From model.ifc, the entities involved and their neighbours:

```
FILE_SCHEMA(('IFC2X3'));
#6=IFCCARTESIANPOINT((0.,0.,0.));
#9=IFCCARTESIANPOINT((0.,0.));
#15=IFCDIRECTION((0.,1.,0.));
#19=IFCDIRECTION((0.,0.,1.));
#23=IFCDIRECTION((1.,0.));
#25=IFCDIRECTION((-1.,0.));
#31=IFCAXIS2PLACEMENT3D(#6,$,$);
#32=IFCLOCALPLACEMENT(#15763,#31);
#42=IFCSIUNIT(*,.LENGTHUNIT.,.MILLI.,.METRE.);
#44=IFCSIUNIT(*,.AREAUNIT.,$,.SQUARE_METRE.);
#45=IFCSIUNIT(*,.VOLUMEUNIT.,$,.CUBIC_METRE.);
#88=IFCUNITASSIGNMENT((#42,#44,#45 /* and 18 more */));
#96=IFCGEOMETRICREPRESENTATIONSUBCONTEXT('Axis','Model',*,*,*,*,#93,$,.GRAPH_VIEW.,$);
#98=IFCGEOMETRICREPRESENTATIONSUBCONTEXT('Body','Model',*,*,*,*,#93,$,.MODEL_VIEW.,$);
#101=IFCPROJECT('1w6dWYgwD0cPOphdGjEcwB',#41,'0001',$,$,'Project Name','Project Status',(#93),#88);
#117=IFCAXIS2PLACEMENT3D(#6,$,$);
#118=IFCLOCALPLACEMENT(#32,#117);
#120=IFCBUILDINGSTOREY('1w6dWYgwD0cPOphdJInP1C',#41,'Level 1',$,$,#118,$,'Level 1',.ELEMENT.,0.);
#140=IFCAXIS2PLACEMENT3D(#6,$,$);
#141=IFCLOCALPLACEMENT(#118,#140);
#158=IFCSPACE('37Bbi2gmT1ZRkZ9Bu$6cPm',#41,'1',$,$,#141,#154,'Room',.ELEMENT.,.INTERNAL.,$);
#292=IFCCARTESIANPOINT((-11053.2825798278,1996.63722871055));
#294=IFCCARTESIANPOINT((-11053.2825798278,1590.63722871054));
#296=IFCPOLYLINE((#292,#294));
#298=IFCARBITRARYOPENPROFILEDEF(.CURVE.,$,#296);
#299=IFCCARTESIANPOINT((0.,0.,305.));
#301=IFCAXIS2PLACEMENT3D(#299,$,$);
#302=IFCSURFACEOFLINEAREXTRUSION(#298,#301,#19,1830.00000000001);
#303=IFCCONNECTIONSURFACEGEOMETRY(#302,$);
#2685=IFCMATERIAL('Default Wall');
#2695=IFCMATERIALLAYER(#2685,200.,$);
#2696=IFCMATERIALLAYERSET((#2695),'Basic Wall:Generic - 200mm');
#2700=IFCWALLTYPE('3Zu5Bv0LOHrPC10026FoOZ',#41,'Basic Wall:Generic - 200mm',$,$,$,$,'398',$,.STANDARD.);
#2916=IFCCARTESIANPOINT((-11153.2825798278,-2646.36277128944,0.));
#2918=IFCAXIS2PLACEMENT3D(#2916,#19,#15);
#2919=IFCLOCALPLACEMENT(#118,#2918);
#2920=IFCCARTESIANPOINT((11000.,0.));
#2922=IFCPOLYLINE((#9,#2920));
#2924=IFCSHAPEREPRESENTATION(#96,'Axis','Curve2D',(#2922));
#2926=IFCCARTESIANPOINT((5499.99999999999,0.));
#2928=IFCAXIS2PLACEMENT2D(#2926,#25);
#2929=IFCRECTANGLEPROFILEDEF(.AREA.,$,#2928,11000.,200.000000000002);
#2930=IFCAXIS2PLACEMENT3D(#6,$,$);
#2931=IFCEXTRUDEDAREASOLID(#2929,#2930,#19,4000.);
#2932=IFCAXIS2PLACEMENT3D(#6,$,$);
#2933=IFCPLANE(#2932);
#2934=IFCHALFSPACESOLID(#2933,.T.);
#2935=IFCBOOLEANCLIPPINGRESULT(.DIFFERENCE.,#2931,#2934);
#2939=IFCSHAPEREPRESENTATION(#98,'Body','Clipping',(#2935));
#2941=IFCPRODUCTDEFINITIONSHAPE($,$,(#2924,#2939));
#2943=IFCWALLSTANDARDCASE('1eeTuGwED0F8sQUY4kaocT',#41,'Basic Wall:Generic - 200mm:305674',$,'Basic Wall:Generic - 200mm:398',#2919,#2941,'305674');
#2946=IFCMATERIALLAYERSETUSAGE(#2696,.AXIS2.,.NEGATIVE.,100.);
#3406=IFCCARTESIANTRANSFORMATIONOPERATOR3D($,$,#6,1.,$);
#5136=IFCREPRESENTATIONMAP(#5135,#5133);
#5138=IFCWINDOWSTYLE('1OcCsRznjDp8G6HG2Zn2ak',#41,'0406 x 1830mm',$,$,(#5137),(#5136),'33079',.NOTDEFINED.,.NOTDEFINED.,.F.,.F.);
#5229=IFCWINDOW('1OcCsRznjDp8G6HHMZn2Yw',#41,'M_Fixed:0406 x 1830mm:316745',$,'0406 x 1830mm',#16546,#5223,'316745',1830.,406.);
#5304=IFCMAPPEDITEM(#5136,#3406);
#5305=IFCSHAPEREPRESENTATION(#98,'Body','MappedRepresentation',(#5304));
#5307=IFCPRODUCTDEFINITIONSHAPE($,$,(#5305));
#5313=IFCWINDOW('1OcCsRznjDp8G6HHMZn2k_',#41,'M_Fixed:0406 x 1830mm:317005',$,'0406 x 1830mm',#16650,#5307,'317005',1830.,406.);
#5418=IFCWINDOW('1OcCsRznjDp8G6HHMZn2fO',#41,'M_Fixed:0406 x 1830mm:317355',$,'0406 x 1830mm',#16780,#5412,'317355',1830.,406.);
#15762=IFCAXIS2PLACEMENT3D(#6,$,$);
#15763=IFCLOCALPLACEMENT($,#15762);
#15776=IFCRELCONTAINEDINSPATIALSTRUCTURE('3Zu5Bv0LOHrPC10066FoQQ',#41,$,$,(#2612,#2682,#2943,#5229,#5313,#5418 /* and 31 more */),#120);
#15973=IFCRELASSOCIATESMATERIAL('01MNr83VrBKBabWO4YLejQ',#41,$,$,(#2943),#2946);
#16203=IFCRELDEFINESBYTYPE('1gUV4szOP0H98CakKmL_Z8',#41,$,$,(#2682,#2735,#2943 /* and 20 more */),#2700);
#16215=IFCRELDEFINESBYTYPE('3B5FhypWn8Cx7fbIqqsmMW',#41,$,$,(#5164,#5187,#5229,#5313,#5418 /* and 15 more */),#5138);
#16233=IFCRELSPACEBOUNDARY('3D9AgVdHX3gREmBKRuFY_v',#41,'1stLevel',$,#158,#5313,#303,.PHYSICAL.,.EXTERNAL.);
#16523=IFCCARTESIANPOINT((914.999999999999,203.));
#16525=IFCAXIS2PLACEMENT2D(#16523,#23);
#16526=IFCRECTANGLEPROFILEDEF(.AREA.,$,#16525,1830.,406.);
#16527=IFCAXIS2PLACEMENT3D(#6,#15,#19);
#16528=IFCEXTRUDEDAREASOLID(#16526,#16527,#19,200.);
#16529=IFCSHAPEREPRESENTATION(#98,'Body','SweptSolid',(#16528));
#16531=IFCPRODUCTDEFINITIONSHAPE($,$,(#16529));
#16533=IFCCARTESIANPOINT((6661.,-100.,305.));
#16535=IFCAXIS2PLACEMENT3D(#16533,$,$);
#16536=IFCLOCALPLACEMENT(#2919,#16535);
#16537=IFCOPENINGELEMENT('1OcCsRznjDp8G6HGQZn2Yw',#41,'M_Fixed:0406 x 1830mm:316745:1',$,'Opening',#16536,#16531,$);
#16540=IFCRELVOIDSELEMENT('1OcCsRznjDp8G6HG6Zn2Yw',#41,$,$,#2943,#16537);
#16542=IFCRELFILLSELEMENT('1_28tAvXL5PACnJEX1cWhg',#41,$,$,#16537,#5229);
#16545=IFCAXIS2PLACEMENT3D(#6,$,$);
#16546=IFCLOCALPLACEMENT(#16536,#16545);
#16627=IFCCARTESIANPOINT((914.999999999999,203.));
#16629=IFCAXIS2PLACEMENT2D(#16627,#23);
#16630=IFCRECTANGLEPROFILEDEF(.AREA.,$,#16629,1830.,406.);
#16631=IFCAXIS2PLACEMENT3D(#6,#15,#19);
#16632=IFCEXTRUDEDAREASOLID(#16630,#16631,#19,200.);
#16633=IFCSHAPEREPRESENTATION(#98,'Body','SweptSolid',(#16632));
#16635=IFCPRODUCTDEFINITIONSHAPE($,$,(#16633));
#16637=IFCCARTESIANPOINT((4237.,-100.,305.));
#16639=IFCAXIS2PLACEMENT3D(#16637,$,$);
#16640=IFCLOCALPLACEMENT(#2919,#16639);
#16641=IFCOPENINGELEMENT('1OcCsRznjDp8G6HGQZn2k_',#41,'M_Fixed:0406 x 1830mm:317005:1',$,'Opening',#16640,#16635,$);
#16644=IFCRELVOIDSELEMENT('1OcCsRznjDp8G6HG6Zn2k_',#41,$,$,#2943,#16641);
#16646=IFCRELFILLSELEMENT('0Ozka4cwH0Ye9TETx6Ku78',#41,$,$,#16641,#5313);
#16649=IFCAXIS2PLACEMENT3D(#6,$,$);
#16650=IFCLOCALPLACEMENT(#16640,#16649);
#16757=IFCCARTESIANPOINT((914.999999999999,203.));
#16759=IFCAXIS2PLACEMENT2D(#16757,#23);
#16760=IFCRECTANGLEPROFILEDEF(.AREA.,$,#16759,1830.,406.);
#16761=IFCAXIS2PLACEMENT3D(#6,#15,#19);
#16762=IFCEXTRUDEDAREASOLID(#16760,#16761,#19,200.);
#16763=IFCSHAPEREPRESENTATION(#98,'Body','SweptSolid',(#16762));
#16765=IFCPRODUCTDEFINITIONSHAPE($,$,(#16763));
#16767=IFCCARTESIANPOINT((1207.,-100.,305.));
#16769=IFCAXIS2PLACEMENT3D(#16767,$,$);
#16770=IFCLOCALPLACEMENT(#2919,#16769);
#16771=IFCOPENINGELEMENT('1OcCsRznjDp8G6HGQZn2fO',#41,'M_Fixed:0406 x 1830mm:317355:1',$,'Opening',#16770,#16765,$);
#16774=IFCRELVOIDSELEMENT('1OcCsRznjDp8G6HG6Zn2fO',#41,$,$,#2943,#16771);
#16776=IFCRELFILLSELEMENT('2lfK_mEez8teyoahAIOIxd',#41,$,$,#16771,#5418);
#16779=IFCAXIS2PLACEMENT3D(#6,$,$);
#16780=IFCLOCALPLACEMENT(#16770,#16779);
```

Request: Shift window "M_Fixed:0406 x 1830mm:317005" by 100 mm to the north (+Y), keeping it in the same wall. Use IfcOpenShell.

```python
import numpy as np
import ifcopenshell
import ifcopenshell.api.geometry
import ifcopenshell.util.placement
import ifcopenshell.util.unit

model = ifcopenshell.open("model.ifc")
unit_scale = ifcopenshell.util.unit.calculate_unit_scale(model)

window = model.by_id(5313)
opening = window.FillsVoids[0].RelatingOpeningElement
wall = opening.VoidsElements[0].RelatingBuildingElement

wall_matrix = ifcopenshell.util.placement.get_local_placement(wall.ObjectPlacement)
shift = wall_matrix[:3, 0] * 0.1 / unit_scale
before = ifcopenshell.util.placement.get_local_placement(window.ObjectPlacement)[:3, 3].copy()

# The window is placed relative to its opening, so it follows when the opening moves.
matrix = ifcopenshell.util.placement.get_local_placement(opening.ObjectPlacement)
matrix[:3, 3] += shift
ifcopenshell.api.geometry.edit_object_placement(
    model, product=opening, matrix=matrix, is_si=False, should_transform_children=True
)

# Space boundary surfaces are stored in each space's coordinates; move them too.
for rel in window.ProvidesBoundaries:
    if not rel.ConnectionGeometry:
        continue
    surface = rel.ConnectionGeometry.SurfaceOnRelatingElement
    space_matrix = ifcopenshell.util.placement.get_local_placement(rel.RelatingSpace.ObjectPlacement)
    point = np.array(surface.Position.Location.Coordinates) + space_matrix[:3, :3].T @ shift
    surface.Position = model.createIfcAxis2Placement3D(
        model.createIfcCartesianPoint(point.tolist()), surface.Position.Axis, surface.Position.RefDirection
    )

after = ifcopenshell.util.placement.get_local_placement(window.ObjectPlacement)[:3, 3]
print("window moved by", (after - before).round(3) + 0.0)

model.write("model-out.ifc")
```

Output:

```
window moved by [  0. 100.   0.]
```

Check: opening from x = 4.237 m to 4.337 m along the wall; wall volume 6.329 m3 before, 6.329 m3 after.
